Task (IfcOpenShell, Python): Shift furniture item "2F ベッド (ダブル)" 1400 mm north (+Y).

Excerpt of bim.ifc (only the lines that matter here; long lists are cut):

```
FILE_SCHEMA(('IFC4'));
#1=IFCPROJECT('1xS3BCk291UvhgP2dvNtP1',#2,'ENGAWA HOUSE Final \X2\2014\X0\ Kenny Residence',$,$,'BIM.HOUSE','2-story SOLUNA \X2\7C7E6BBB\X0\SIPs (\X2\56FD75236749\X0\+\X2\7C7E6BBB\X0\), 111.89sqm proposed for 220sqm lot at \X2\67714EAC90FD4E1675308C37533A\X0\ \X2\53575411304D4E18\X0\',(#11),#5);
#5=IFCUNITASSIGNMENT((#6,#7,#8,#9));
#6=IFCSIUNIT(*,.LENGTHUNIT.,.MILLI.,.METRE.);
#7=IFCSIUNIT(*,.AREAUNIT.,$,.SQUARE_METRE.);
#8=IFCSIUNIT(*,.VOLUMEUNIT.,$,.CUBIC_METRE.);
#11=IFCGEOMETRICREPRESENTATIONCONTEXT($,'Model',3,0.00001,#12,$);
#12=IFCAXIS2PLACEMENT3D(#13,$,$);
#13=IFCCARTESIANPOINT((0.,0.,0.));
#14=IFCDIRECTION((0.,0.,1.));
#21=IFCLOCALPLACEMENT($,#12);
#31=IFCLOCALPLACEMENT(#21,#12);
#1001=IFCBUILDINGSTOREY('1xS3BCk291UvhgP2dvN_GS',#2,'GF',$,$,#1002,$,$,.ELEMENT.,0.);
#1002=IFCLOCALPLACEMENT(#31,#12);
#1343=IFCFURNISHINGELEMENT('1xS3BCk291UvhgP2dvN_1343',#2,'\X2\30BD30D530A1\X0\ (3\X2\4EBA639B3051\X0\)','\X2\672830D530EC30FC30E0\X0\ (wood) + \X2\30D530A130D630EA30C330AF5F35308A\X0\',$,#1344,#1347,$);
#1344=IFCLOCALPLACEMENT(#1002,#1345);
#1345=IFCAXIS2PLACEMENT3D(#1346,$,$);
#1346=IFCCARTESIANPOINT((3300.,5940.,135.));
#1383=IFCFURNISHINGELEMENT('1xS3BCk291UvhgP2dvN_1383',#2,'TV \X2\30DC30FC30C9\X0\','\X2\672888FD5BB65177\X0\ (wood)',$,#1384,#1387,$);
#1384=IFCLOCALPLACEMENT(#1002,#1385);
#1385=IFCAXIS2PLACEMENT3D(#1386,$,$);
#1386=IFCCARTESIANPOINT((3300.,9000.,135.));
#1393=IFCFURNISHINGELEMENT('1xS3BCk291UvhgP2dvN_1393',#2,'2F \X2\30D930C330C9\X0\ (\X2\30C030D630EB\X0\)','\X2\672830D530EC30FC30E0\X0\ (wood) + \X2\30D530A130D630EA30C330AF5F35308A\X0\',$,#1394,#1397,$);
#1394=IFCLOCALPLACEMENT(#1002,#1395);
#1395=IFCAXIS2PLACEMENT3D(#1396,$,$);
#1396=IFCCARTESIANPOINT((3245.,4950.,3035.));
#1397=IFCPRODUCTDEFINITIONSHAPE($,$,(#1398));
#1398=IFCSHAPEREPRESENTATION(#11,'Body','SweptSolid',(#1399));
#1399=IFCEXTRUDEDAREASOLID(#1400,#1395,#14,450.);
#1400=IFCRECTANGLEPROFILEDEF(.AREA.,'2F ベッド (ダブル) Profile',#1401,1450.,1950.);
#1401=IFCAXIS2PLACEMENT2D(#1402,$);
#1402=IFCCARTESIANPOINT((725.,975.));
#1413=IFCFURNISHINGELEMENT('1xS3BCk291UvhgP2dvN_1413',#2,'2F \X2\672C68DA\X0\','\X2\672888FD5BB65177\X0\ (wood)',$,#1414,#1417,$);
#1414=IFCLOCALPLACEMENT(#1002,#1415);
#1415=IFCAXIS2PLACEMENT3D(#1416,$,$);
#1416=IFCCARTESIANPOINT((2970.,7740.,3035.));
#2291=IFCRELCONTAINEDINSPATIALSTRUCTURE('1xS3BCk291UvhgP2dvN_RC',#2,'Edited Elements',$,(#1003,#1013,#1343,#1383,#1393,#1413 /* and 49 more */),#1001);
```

```python
import ifcopenshell
import ifcopenshell.api.geometry
import ifcopenshell.util.placement

model = ifcopenshell.open("bim.ifc")

item = model.by_id(1393)
matrix = ifcopenshell.util.placement.get_local_placement(item.ObjectPlacement)
matrix[1, 3] += 1400.0
ifcopenshell.api.geometry.edit_object_placement(model, product=item, matrix=matrix, is_si=False)

print(ifcopenshell.util.placement.get_local_placement(item.ObjectPlacement).round(3) + 0.0)

model.write("bim_updated.ifc")
```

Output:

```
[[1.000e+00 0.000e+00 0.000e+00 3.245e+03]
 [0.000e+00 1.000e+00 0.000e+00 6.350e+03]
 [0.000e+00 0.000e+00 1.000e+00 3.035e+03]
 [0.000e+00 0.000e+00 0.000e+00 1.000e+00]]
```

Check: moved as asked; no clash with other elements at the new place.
